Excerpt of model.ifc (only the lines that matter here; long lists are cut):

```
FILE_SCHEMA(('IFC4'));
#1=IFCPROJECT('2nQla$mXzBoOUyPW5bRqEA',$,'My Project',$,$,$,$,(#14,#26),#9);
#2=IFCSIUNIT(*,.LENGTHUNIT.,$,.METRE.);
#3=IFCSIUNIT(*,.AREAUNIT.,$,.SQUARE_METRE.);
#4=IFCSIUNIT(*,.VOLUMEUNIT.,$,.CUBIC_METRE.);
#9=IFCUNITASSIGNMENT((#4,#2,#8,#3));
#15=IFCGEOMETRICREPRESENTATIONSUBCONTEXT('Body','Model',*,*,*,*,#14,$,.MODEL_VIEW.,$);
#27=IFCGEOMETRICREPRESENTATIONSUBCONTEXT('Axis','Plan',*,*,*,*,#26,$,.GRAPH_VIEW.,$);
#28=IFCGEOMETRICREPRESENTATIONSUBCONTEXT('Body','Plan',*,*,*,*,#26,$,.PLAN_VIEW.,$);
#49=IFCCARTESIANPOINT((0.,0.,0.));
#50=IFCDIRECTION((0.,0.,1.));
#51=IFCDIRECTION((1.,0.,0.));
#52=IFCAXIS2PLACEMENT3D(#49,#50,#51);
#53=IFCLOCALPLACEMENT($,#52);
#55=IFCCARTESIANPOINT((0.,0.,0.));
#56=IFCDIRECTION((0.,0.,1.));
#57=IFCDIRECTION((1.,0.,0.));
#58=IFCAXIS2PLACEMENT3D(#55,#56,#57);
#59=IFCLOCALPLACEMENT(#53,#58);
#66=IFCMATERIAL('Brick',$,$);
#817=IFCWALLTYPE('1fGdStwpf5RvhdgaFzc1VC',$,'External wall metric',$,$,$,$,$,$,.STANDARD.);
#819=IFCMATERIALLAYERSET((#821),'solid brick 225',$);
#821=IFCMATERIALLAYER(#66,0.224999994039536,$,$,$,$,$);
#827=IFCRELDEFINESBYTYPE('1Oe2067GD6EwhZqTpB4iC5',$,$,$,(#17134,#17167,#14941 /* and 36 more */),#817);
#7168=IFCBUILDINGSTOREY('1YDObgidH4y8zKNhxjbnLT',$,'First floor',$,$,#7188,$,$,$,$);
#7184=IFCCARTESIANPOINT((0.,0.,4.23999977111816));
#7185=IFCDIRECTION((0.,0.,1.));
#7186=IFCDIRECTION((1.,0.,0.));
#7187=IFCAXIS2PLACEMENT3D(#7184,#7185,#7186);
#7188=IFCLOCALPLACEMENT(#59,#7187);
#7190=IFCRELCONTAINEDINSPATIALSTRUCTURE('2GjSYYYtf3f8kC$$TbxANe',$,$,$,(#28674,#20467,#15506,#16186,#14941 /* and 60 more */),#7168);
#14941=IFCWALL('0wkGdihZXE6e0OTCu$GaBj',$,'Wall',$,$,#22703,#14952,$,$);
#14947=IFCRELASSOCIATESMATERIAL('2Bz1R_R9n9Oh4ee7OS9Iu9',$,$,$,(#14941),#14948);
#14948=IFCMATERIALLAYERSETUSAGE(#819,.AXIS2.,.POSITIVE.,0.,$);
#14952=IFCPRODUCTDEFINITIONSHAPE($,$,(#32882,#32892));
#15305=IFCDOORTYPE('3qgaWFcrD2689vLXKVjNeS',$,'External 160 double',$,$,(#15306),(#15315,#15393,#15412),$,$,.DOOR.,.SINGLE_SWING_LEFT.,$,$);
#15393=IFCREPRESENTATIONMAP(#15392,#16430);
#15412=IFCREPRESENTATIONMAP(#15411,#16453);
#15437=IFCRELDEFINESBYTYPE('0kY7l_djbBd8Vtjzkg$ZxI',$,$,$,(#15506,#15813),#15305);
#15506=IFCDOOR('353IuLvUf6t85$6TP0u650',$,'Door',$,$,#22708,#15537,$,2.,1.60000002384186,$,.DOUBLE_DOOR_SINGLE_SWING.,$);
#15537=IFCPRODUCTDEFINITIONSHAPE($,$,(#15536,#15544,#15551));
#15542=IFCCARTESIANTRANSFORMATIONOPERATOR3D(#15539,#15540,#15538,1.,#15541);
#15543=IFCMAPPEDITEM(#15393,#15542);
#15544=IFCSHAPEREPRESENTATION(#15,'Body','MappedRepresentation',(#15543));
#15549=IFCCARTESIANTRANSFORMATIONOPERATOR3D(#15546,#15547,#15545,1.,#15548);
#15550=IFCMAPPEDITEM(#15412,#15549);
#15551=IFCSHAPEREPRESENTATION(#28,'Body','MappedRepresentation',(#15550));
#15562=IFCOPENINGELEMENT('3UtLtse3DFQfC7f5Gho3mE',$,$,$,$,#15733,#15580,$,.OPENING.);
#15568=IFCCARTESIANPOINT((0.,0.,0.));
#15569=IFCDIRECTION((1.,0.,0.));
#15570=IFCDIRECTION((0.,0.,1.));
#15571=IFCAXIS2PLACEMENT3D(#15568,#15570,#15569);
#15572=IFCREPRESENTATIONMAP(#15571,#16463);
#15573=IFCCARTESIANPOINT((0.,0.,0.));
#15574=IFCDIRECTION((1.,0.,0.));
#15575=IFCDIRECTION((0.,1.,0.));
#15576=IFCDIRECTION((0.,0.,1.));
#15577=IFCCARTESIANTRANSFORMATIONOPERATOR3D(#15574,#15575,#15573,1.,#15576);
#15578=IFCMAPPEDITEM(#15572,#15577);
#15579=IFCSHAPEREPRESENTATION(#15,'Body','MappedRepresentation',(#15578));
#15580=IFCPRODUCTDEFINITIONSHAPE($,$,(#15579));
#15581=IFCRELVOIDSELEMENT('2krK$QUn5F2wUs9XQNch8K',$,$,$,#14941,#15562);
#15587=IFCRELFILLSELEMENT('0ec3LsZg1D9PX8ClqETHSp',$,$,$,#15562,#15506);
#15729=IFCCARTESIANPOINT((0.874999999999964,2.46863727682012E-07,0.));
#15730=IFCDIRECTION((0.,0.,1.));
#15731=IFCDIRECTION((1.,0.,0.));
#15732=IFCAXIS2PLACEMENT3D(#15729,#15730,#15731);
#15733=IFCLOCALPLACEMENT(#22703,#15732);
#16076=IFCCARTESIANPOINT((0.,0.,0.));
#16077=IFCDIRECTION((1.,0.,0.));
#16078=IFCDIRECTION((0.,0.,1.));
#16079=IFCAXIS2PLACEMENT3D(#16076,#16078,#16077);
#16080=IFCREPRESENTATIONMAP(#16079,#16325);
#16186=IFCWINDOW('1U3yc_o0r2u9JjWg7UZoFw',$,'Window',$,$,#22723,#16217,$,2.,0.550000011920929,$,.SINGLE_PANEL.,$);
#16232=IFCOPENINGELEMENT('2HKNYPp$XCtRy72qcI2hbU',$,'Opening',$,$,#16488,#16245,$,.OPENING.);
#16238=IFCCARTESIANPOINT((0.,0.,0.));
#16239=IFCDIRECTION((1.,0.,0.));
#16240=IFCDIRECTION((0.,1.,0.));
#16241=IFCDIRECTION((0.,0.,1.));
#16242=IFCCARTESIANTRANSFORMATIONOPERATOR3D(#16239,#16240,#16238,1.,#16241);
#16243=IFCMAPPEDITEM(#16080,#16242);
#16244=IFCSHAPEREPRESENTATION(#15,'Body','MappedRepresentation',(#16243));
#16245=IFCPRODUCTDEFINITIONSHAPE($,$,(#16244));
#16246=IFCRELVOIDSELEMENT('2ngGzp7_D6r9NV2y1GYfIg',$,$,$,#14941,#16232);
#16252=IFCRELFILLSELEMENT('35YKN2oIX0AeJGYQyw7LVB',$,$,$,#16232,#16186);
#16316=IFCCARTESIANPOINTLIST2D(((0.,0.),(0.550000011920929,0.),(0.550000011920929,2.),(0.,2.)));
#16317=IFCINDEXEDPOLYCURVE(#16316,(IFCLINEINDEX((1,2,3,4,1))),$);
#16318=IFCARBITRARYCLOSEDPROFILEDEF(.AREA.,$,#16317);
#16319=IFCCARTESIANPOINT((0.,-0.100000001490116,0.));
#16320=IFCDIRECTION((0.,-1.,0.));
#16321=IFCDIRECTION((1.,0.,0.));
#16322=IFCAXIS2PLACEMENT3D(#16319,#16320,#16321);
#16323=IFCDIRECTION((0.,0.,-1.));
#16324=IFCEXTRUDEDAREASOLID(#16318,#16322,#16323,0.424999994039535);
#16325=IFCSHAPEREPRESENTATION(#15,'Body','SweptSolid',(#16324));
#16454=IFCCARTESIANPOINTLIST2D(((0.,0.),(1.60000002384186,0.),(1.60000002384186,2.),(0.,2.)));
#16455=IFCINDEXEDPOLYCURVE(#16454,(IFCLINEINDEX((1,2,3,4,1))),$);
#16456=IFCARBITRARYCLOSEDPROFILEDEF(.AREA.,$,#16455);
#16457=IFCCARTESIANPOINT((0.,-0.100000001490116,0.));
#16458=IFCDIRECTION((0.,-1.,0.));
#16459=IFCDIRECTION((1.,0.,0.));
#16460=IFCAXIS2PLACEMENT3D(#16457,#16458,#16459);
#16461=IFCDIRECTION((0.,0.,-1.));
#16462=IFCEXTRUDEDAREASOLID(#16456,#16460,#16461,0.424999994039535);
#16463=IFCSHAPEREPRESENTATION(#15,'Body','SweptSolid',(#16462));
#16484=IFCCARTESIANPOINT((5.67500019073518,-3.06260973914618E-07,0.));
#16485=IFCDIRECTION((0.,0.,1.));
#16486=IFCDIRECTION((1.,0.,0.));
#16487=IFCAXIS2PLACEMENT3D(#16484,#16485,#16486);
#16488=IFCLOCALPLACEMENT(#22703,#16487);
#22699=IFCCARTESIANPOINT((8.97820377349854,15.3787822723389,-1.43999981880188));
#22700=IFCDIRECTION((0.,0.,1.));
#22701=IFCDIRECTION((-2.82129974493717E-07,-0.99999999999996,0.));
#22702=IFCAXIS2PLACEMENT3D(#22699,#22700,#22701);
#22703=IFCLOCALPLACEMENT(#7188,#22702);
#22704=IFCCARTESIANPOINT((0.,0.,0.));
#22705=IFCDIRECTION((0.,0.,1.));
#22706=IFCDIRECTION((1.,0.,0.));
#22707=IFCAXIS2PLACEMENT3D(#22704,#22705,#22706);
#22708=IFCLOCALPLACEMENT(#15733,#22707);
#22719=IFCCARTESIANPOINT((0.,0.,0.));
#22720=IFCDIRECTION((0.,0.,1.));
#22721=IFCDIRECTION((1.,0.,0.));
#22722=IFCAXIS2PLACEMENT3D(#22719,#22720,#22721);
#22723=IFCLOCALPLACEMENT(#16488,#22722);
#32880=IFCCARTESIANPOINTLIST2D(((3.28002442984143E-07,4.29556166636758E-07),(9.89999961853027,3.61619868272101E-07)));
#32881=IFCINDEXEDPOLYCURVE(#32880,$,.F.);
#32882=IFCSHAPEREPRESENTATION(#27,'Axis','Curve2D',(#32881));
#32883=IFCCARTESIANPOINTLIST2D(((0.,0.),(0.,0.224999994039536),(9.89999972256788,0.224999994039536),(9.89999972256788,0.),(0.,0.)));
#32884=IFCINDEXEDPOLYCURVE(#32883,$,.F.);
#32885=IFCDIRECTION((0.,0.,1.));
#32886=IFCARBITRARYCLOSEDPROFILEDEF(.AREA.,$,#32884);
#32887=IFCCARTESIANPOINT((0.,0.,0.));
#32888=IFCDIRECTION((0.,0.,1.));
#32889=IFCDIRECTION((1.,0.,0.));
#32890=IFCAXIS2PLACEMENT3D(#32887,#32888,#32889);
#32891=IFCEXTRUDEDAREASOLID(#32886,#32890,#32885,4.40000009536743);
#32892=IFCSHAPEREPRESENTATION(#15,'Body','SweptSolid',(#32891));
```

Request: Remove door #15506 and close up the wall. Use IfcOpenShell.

```python
import ifcopenshell
import ifcopenshell.api.feature
import ifcopenshell.api.root
import ifcopenshell.geom
import ifcopenshell.util.shape

model = ifcopenshell.open("model.ifc")
settings = ifcopenshell.geom.settings()


def volume(element):
    """Net volume in cubic metres, openings subtracted."""
    shape = ifcopenshell.geom.create_shape(settings, element)
    return ifcopenshell.util.shape.get_volume(shape.geometry)


door = model.by_guid("353IuLvUf6t85$6TP0u650")
opening = door.FillsVoids[0].RelatingOpeningElement
wall = opening.VoidsElements[0].RelatingBuildingElement
before = volume(wall)

ifcopenshell.api.root.remove_product(model, product=door)
ifcopenshell.api.feature.remove_feature(model, feature=opening)

after = volume(wall)

print(f"wall volume {before:.3f} -> {after:.3f} m3")

model.write("model_rev.ifc")
```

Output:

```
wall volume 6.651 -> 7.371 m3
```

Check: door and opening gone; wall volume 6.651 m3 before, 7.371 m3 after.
